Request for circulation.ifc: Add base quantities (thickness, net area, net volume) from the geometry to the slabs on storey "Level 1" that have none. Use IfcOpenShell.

First a look at what the model holds.

```python
import ifcopenshell
import ifcopenshell.util.element
import ifcopenshell.util.unit

model = ifcopenshell.open("circulation.ifc")
print(model.schema)
for unit_type in ("LENGTHUNIT", "AREAUNIT", "VOLUMEUNIT"):
    print(unit_type, ifcopenshell.util.unit.calculate_unit_scale(model, unit_type))
storey = next(s for s in model.by_type("IfcBuildingStorey") if s.Name == "Level 1")
slabs = [e for e in ifcopenshell.util.element.get_decomposition(storey) if e.is_a("IfcSlab")]
for e in sorted(slabs, key=lambda e: e.id()):
    print(e.id(), e.is_a(), e.Name, list(ifcopenshell.util.element.get_psets(e, qtos_only=True)), sep=" | ")
```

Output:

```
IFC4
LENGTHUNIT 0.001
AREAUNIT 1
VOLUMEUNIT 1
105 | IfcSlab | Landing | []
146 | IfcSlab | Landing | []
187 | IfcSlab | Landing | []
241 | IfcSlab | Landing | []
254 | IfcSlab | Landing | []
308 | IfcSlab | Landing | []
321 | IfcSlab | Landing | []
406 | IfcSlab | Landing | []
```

```python
import ifcopenshell
import ifcopenshell.api.pset
import ifcopenshell.geom
import ifcopenshell.util.element
import ifcopenshell.util.shape
import ifcopenshell.util.unit

model = ifcopenshell.open("circulation.ifc")
unit_scale = ifcopenshell.util.unit.calculate_unit_scale(model)
area_scale = ifcopenshell.util.unit.calculate_unit_scale(model, "AREAUNIT")
volume_scale = ifcopenshell.util.unit.calculate_unit_scale(model, "VOLUMEUNIT")
settings = ifcopenshell.geom.settings()

storey = next(s for s in model.by_type("IfcBuildingStorey") if s.Name == "Level 1")
slabs = [e for e in ifcopenshell.util.element.get_decomposition(storey) if e.is_a("IfcSlab")]

for e in sorted(slabs, key=lambda e: e.id()):
    if ifcopenshell.util.element.get_psets(e, qtos_only=True, should_inherit=False):
        continue
    # Geometry comes back in metres, in the element's own axes.
    shape = ifcopenshell.geom.create_shape(settings, e)
    values = {
        "Width": ifcopenshell.util.shape.get_z(shape.geometry) / unit_scale,
        "NetArea": ifcopenshell.util.shape.get_footprint_area(shape.geometry) / area_scale,
        "NetVolume": ifcopenshell.util.shape.get_volume(shape.geometry) / volume_scale,
    }
    qto = ifcopenshell.api.pset.add_qto(model, product=e, name="Qto_SlabBaseQuantities")
    ifcopenshell.api.pset.edit_qto(model, qto=qto, properties=values)
    print(e.id(), {k: round(v, 3) for k, v in values.items()})

model.write("circulation_edited.ifc")
```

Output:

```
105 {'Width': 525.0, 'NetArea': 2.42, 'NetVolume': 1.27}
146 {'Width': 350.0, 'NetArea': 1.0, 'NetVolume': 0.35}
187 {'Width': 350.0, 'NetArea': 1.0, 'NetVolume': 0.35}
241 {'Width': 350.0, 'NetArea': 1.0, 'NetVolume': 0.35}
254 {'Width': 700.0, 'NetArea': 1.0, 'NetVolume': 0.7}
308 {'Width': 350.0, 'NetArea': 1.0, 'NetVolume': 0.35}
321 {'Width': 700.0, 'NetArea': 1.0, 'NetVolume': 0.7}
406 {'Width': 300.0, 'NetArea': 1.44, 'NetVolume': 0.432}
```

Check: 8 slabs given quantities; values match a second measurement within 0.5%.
